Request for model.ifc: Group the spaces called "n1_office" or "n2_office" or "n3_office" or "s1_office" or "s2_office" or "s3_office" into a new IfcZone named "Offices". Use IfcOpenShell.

First a look at what the model holds.

```python
import ifcopenshell

model = ifcopenshell.open("model.ifc")
print(model.schema)
seen = {}
for space in model.by_type("IfcSpace"):
    seen[space.Name] = seen.get(space.Name, 0) + 1
for name, count in sorted(seen.items(), key=str):
    print(count, "x", name)
print("zones:", [z.Name for z in model.by_type("IfcZone")][:20])
```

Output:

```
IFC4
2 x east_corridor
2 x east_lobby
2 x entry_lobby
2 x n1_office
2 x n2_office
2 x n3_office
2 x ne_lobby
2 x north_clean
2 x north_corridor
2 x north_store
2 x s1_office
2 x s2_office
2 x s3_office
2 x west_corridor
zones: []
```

```python
import ifcopenshell
import ifcopenshell.api.group
import ifcopenshell.api.root

model = ifcopenshell.open("model.ifc")

names = {"n1_office", "n2_office", "n3_office", "s1_office", "s2_office", "s3_office"}
spaces = [s for s in model.by_type("IfcSpace") if s.Name in names]

zone = ifcopenshell.api.root.create_entity(model, ifc_class="IfcZone", name="Offices")
ifcopenshell.api.group.assign_group(model, products=spaces, group=zone)
print(len(spaces), "spaces in", zone.Name)

model.write("model_edited.ifc")
```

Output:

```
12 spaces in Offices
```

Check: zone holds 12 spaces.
